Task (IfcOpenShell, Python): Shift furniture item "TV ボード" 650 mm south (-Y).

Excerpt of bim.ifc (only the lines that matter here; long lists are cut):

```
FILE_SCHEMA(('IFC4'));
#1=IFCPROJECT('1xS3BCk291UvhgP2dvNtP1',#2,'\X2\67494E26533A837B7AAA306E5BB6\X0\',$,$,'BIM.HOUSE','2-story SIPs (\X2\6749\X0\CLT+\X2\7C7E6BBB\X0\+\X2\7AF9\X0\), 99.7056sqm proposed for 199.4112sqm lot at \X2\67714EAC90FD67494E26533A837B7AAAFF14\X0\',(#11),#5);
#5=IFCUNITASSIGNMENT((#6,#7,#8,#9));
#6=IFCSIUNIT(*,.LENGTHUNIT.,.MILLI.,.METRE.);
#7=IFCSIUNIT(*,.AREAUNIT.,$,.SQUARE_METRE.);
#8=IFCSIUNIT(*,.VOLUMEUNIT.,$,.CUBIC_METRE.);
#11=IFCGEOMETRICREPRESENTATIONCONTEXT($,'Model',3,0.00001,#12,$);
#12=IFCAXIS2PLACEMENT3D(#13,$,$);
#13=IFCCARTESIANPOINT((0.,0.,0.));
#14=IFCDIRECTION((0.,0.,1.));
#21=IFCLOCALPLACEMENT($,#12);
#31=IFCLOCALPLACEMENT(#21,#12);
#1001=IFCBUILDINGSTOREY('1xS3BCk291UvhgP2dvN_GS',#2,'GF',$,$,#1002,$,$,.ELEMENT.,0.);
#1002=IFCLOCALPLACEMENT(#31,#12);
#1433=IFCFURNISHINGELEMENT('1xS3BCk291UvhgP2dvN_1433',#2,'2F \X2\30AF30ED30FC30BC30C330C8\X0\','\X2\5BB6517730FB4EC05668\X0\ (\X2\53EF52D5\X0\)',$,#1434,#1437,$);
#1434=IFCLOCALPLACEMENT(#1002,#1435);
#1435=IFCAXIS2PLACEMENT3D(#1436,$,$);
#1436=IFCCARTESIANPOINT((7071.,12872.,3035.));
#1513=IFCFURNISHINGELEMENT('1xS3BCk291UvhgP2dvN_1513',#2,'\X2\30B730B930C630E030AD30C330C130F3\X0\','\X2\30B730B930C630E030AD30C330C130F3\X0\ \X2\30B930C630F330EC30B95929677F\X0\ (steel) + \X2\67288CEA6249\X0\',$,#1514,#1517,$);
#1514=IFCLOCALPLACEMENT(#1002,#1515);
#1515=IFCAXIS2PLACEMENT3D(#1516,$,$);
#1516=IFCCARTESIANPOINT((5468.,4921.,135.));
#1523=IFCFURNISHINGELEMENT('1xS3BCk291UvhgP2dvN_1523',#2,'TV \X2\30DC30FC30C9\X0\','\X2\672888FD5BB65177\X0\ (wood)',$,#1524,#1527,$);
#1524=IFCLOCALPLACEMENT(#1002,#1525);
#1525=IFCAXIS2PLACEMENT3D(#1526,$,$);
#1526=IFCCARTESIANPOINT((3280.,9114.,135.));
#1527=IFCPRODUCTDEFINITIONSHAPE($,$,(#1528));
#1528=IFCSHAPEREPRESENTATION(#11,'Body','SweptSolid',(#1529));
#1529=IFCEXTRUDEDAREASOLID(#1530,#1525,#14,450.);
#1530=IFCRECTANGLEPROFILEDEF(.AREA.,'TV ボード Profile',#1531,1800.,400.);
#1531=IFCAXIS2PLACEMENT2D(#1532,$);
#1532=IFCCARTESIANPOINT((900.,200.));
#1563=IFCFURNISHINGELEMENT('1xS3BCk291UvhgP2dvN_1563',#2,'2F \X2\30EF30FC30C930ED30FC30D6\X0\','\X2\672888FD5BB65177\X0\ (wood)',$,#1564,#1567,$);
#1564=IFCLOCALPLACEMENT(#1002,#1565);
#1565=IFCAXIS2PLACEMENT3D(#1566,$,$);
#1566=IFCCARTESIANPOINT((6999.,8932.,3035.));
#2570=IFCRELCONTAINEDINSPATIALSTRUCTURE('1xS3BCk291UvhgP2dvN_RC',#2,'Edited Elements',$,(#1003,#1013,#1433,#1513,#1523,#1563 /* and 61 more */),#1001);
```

```python
import ifcopenshell
import ifcopenshell.api.geometry
import ifcopenshell.util.placement
import ifcopenshell.util.unit

model = ifcopenshell.open("bim.ifc")
unit_scale = ifcopenshell.util.unit.calculate_unit_scale(model)

item = model.by_id(1523)
matrix = ifcopenshell.util.placement.get_local_placement(item.ObjectPlacement)
matrix[1, 3] -= 0.65 / unit_scale
ifcopenshell.api.geometry.edit_object_placement(model, product=item, matrix=matrix, is_si=False)

print(ifcopenshell.util.placement.get_local_placement(item.ObjectPlacement).round(3) + 0.0)

model.write("bim_updated.ifc")
```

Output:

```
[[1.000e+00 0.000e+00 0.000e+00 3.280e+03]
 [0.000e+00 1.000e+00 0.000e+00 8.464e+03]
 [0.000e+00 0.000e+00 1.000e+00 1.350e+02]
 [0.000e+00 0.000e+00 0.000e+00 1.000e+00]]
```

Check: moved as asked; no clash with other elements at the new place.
